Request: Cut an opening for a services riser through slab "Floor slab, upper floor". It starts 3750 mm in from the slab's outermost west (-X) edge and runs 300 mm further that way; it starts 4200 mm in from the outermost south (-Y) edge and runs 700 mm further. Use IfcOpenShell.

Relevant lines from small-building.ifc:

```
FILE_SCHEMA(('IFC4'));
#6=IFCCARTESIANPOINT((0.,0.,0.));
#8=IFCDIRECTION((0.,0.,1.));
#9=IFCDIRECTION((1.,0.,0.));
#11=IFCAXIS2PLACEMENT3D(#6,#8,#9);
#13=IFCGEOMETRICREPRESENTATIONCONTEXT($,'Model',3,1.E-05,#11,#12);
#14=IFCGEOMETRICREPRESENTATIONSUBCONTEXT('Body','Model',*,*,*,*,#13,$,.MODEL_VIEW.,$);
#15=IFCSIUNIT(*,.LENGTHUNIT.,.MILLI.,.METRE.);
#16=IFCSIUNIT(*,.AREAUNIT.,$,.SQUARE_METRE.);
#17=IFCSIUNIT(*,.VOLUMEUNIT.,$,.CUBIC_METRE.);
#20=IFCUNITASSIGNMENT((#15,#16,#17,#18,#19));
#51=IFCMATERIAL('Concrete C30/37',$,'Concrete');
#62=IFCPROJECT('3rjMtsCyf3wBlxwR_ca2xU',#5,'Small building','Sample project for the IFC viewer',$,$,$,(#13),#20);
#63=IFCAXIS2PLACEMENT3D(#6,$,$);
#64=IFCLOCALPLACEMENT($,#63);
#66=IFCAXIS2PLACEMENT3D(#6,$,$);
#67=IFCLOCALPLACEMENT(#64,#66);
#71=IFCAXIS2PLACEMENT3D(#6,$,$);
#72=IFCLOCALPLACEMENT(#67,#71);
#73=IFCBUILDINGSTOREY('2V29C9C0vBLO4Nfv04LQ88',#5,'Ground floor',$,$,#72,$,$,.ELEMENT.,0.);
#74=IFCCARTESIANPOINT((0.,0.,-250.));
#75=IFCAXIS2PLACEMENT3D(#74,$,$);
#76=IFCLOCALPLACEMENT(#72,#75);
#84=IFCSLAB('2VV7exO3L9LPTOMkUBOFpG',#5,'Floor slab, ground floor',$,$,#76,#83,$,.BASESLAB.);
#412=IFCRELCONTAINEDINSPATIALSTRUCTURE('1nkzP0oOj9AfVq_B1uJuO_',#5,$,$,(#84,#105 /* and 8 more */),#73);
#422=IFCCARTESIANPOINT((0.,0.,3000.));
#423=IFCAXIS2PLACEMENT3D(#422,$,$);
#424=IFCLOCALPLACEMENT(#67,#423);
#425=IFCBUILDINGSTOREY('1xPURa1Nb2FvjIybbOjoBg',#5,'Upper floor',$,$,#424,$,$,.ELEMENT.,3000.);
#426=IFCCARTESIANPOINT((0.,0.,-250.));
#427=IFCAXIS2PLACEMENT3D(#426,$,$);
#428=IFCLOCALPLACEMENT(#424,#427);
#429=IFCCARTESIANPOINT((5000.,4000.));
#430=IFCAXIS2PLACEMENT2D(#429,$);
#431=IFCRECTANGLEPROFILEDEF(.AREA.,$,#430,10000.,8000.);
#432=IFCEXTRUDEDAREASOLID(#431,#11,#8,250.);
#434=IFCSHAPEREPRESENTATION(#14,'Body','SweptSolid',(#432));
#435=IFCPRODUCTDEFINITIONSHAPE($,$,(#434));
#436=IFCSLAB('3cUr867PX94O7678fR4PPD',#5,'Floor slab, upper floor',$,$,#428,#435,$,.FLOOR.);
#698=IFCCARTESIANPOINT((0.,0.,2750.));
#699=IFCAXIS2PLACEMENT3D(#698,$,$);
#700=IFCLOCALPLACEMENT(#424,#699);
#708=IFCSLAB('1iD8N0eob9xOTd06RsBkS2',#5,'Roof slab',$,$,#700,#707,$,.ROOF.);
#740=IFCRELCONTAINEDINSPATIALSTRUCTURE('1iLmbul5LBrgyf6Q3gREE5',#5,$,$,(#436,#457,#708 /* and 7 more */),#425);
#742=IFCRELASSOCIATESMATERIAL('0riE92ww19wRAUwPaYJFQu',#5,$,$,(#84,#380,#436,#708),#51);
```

```python
import numpy as np
import ifcopenshell
import ifcopenshell.api.feature
import ifcopenshell.api.geometry
import ifcopenshell.api.root
import ifcopenshell.geom
import ifcopenshell.util.placement
import ifcopenshell.util.representation
import ifcopenshell.util.shape
import ifcopenshell.util.unit

model = ifcopenshell.open("small-building.ifc")
unit_scale = ifcopenshell.util.unit.calculate_unit_scale(model)
settings = ifcopenshell.geom.settings()


def volume(element):
    """Net volume in cubic metres, openings subtracted."""
    shape = ifcopenshell.geom.create_shape(settings, element)
    return ifcopenshell.util.shape.get_volume(shape.geometry)


slab = model.by_id(436)
before = volume(slab)

# Extent in the slab's own axes, in metres. The edges named are its -X and -Y sides.
slab_shape = ifcopenshell.geom.create_shape(settings, slab)
vertices = ifcopenshell.util.shape.get_vertices(slab_shape.geometry)
x_min, y_min, bottom = vertices.min(axis=0)
top = vertices[:, 2].max()

opening = ifcopenshell.api.root.create_entity(model, ifc_class="IfcOpeningElement", name="Services riser opening", predefined_type="OPENING")
context = ifcopenshell.util.representation.get_context(model, "Model", "Body", "MODEL_VIEW")
width, depth = 0.3, 0.7
outline = [(0.0, 0.0), (width, 0.0), (width, depth), (0.0, depth), (0.0, 0.0)]
# Overshoot both faces by 50 mm so the cut is clean.
shape = ifcopenshell.api.geometry.add_slab_representation(
    model, context=context, depth=top - bottom + 0.1, polyline=outline
)
ifcopenshell.api.geometry.assign_representation(model, product=opening, representation=shape)

matrix = ifcopenshell.util.placement.get_local_placement(slab.ObjectPlacement)
matrix[:, 3] = matrix @ np.append(np.array([x_min + 3.75, y_min + 4.2, bottom - 0.05]) / unit_scale, 1.0)
ifcopenshell.api.geometry.edit_object_placement(model, product=opening, matrix=matrix, is_si=False)
ifcopenshell.api.feature.add_feature(model, feature=opening, element=slab)

after = volume(slab)

print(f"slab volume {before:.3f} -> {after:.3f} m3")

model.write("small-building_rev.ifc")
```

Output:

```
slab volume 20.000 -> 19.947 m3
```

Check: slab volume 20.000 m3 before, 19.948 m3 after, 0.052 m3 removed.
